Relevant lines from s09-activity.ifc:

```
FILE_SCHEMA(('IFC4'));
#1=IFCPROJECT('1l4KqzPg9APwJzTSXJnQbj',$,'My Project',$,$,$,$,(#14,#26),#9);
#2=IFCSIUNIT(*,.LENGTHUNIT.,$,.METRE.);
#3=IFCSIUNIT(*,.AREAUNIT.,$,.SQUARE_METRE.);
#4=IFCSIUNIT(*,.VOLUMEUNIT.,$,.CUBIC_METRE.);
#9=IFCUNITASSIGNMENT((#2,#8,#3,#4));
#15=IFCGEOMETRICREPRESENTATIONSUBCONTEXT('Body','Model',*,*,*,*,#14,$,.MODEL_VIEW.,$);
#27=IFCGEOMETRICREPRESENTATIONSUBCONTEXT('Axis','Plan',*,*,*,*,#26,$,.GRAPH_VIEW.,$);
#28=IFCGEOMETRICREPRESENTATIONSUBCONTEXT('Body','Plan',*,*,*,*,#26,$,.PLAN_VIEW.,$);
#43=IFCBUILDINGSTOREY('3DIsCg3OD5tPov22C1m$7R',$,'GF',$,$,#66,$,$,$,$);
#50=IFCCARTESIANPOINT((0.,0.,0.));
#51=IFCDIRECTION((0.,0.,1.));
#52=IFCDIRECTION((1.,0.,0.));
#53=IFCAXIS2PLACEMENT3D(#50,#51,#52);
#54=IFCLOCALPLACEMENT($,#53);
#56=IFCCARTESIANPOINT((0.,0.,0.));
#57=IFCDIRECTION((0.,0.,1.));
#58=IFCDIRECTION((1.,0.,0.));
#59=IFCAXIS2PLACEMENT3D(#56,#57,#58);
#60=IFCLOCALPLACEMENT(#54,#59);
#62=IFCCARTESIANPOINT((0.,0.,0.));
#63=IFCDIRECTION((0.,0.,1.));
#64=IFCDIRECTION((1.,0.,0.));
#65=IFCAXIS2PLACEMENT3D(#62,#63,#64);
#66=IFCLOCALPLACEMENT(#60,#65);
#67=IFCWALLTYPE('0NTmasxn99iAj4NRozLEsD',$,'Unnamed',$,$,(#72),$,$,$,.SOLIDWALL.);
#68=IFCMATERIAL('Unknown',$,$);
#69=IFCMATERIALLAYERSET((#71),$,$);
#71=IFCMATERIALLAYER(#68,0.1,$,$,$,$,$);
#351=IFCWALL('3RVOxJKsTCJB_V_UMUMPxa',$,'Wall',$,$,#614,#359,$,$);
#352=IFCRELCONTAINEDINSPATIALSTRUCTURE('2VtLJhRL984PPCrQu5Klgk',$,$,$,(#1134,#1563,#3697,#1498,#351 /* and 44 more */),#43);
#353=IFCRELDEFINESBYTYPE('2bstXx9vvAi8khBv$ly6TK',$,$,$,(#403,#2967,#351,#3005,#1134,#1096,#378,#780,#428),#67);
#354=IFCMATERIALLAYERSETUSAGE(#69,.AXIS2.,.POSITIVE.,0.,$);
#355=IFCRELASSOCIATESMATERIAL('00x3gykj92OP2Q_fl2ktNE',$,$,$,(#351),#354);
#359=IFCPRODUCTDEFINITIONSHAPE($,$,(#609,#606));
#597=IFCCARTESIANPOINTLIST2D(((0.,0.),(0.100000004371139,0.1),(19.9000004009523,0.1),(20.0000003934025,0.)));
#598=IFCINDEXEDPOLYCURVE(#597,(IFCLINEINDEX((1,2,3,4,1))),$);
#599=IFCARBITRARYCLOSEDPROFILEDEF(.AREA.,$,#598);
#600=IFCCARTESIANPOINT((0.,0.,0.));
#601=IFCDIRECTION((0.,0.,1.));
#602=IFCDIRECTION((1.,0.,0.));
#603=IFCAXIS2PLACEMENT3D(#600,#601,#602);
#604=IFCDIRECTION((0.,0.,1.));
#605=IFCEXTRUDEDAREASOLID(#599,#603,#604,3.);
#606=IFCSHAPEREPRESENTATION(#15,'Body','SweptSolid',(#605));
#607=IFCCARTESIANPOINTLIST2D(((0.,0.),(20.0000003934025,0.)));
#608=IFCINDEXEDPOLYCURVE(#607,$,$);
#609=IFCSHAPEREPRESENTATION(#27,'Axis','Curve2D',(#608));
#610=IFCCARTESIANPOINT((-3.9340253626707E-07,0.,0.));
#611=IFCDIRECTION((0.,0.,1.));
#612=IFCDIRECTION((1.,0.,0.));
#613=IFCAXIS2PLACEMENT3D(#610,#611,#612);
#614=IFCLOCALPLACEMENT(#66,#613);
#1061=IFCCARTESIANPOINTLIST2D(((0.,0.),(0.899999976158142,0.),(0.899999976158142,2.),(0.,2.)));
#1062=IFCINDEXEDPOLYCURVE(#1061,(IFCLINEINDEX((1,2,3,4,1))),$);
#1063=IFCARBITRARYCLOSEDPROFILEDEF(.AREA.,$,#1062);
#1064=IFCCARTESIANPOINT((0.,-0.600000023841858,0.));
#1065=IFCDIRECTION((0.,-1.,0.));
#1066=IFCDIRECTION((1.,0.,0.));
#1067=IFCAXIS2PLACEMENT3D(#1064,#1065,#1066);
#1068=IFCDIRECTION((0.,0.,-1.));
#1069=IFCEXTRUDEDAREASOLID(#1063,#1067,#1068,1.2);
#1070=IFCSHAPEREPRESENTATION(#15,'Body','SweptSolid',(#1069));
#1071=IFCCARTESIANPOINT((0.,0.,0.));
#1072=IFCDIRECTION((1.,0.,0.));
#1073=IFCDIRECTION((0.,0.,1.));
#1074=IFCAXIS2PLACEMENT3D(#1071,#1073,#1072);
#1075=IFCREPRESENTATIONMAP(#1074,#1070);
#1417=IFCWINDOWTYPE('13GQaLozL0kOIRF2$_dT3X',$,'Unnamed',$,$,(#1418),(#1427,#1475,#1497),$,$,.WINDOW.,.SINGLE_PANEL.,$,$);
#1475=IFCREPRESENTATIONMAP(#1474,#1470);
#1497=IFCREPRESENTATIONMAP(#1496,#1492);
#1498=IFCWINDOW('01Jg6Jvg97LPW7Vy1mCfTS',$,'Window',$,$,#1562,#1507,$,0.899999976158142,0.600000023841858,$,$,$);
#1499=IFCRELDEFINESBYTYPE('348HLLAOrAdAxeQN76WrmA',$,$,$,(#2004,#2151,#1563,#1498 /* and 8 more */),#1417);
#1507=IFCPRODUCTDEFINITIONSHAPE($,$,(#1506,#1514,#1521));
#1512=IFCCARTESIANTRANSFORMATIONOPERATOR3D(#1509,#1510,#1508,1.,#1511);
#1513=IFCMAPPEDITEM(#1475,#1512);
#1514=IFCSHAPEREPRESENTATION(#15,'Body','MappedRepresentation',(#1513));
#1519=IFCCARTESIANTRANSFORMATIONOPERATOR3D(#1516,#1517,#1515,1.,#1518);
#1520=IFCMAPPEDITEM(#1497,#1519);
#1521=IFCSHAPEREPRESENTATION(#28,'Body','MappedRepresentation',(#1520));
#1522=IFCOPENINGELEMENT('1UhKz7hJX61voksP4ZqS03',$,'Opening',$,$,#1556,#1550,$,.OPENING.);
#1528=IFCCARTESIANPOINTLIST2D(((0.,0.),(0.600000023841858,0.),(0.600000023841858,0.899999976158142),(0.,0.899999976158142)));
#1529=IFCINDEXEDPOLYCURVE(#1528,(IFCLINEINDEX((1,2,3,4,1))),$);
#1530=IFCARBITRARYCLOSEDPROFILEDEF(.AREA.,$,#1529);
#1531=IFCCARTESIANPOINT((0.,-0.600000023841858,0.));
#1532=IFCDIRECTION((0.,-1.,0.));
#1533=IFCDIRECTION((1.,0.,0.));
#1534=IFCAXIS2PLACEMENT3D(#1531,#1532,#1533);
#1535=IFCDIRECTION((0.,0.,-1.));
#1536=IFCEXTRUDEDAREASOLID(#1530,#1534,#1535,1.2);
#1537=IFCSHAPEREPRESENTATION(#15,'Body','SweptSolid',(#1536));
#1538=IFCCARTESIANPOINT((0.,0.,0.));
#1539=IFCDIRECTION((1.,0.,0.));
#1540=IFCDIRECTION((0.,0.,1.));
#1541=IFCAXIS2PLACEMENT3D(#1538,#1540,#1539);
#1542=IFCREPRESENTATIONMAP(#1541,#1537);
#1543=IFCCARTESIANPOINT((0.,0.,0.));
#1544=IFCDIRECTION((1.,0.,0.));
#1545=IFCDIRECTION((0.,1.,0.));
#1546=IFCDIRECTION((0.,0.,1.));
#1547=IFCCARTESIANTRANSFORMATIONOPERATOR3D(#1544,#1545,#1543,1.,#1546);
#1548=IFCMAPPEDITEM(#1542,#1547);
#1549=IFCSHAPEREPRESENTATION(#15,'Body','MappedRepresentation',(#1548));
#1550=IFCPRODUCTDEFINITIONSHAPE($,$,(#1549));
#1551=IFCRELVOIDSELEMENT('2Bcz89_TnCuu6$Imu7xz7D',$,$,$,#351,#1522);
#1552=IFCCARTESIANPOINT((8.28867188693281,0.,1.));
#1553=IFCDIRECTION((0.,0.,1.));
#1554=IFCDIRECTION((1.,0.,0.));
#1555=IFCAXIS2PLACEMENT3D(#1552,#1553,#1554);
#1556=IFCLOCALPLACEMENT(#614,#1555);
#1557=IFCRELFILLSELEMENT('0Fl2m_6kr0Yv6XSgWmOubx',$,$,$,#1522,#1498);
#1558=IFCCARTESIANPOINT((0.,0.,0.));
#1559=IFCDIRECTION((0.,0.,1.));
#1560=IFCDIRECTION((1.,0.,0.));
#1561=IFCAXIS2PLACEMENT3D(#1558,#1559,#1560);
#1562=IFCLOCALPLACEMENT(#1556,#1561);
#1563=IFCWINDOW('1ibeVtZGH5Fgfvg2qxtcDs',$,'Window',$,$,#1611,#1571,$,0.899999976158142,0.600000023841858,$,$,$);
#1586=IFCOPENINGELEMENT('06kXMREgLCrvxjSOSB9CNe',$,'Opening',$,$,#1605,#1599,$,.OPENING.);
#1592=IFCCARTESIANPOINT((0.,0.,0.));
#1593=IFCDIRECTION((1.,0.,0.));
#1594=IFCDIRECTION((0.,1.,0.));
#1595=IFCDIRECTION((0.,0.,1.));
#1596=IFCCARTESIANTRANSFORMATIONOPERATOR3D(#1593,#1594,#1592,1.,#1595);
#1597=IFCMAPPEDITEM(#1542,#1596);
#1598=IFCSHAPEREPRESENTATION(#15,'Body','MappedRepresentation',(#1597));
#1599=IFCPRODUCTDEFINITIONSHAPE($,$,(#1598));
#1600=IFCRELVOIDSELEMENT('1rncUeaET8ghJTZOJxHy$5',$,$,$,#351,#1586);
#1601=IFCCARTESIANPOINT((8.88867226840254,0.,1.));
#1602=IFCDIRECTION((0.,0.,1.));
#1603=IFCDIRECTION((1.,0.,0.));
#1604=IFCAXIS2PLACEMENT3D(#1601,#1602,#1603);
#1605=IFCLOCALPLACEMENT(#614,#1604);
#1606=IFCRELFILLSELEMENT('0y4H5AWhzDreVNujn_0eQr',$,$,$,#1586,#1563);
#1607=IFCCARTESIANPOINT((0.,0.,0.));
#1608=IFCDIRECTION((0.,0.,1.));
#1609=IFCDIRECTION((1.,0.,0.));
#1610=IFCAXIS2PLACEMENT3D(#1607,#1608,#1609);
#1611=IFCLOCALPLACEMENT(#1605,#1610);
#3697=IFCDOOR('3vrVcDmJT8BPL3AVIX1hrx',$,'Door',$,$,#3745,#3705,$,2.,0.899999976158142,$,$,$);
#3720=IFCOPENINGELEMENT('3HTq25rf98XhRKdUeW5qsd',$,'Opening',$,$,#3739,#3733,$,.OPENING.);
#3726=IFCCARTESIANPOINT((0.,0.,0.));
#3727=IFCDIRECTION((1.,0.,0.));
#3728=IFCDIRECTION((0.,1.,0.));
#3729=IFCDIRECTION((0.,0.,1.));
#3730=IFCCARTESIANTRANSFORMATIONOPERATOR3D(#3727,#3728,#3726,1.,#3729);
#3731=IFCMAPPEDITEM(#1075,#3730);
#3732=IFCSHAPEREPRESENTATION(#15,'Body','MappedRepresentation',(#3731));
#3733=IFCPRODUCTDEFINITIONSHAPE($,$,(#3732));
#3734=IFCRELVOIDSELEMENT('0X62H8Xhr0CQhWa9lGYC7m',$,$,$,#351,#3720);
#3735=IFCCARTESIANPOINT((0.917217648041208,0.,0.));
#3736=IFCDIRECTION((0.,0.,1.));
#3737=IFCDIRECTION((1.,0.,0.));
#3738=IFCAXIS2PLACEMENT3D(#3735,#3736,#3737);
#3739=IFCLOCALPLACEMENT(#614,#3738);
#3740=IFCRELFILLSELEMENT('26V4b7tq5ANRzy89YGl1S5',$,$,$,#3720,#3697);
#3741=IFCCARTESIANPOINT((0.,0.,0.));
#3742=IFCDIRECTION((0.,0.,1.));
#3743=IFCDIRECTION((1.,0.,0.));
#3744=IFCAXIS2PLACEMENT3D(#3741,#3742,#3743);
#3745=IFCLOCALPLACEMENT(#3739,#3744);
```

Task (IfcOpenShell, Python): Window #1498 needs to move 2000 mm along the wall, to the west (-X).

```python
import ifcopenshell
import ifcopenshell.api.geometry
import ifcopenshell.util.placement

model = ifcopenshell.open("s09-activity.ifc")

window = model.by_guid("01Jg6Jvg97LPW7Vy1mCfTS")
opening = window.FillsVoids[0].RelatingOpeningElement
wall = opening.VoidsElements[0].RelatingBuildingElement

wall_matrix = ifcopenshell.util.placement.get_local_placement(wall.ObjectPlacement)
shift = wall_matrix[:3, 0] * -2.0
before = ifcopenshell.util.placement.get_local_placement(window.ObjectPlacement)[:3, 3].copy()

# The window is placed relative to its opening, so it follows when the opening moves.
matrix = ifcopenshell.util.placement.get_local_placement(opening.ObjectPlacement)
matrix[:3, 3] += shift
ifcopenshell.api.geometry.edit_object_placement(
    model, product=opening, matrix=matrix, is_si=False, should_transform_children=True
)

after = ifcopenshell.util.placement.get_local_placement(window.ObjectPlacement)[:3, 3]
print("window moved by", (after - before).round(3) + 0.0)

model.write("s09-activity_edited.ifc")
```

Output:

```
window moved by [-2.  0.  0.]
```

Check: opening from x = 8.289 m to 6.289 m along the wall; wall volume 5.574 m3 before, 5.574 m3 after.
